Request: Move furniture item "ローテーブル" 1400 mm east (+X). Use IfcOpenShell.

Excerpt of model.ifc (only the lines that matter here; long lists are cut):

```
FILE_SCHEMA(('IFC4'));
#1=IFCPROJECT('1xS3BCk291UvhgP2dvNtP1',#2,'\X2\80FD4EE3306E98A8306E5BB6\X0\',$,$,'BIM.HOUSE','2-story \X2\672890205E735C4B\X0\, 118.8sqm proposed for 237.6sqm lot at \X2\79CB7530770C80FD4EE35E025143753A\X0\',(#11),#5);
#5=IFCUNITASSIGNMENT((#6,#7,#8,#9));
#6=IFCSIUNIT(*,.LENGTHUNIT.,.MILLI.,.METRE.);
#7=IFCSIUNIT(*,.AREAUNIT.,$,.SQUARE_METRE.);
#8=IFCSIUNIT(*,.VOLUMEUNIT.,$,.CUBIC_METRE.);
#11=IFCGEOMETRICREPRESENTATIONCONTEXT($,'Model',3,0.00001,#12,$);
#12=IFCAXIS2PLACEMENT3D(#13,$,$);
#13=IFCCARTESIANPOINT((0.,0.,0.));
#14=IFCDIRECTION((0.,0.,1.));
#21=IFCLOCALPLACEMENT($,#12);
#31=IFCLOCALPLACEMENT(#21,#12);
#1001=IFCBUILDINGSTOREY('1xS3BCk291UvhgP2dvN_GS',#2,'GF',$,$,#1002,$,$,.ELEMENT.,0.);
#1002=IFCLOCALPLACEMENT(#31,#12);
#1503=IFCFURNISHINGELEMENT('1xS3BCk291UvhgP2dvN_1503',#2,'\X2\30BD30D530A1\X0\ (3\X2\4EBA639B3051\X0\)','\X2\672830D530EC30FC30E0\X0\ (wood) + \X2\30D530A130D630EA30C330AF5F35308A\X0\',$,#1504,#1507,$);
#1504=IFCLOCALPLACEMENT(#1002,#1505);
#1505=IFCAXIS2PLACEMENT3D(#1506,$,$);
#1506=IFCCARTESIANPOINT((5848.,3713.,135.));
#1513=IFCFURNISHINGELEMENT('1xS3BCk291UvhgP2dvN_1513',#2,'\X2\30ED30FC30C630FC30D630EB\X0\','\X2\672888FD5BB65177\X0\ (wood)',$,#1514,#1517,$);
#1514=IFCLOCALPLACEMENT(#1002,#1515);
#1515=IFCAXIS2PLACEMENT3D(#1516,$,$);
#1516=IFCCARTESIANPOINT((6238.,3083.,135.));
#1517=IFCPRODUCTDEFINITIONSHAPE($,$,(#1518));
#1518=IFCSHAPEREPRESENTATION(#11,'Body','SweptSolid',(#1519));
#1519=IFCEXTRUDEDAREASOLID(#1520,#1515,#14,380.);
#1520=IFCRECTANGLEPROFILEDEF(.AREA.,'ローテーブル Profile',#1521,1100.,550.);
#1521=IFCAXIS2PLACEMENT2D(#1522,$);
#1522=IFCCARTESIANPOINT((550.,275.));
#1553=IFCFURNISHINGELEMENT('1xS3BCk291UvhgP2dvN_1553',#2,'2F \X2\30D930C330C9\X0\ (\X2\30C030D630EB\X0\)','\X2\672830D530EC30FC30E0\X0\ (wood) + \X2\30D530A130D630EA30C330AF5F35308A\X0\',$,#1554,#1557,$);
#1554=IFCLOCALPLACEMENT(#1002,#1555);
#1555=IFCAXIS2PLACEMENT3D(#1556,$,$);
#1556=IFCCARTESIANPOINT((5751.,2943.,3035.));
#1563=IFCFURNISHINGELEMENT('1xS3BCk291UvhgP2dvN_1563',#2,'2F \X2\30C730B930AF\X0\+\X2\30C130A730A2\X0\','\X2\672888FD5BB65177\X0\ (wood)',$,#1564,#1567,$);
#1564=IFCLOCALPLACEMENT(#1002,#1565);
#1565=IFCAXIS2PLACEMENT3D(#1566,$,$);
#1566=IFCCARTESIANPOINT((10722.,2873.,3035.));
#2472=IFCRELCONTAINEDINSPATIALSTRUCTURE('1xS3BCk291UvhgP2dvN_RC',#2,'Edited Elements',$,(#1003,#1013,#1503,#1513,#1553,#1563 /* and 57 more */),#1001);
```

```python
import ifcopenshell
import ifcopenshell.api.geometry
import ifcopenshell.util.placement
import ifcopenshell.util.unit

model = ifcopenshell.open("model.ifc")
unit_scale = ifcopenshell.util.unit.calculate_unit_scale(model)

item = model.by_guid("1xS3BCk291UvhgP2dvN_1513")
matrix = ifcopenshell.util.placement.get_local_placement(item.ObjectPlacement)
matrix[0, 3] += 1.4 / unit_scale
ifcopenshell.api.geometry.edit_object_placement(model, product=item, matrix=matrix, is_si=False)

print(ifcopenshell.util.placement.get_local_placement(item.ObjectPlacement).round(3) + 0.0)

model.write("model_v2.ifc")
```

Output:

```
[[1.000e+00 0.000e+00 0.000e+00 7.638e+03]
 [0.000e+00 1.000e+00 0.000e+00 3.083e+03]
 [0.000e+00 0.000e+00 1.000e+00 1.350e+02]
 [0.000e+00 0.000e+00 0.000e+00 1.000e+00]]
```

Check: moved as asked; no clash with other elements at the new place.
